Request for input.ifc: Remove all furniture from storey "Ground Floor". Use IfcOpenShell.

First a look at what the model holds.

```python
import ifcopenshell
import ifcopenshell.util.element

model = ifcopenshell.open("input.ifc")
print(model.schema)
storey = next(s for s in model.by_type("IfcBuildingStorey") if s.Name == "Ground Floor")
furniture = [e for e in ifcopenshell.util.element.get_decomposition(storey) if e.is_a("IfcFurnishingElement")]
seen = {}
for e in furniture:
    element_type = ifcopenshell.util.element.get_type(e)
    name = element_type.Name if element_type not in (None, e) else None
    seen[name] = seen.get(name, 0) + 1
for name, count in sorted(seen.items(), key=str):
    print(count, "x", name)
```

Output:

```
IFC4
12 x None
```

```python
import ifcopenshell
import ifcopenshell.api.root
import ifcopenshell.util.element

model = ifcopenshell.open("input.ifc")

storey = next(s for s in model.by_type("IfcBuildingStorey") if s.Name == "Ground Floor")
furniture = [e for e in ifcopenshell.util.element.get_decomposition(storey) if e.is_a("IfcFurnishingElement")]

for e in furniture:
    ifcopenshell.api.root.remove_product(model, product=e)
print(len(furniture), "removed")

model.write("input_v2.ifc")
```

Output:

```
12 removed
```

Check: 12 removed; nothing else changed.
